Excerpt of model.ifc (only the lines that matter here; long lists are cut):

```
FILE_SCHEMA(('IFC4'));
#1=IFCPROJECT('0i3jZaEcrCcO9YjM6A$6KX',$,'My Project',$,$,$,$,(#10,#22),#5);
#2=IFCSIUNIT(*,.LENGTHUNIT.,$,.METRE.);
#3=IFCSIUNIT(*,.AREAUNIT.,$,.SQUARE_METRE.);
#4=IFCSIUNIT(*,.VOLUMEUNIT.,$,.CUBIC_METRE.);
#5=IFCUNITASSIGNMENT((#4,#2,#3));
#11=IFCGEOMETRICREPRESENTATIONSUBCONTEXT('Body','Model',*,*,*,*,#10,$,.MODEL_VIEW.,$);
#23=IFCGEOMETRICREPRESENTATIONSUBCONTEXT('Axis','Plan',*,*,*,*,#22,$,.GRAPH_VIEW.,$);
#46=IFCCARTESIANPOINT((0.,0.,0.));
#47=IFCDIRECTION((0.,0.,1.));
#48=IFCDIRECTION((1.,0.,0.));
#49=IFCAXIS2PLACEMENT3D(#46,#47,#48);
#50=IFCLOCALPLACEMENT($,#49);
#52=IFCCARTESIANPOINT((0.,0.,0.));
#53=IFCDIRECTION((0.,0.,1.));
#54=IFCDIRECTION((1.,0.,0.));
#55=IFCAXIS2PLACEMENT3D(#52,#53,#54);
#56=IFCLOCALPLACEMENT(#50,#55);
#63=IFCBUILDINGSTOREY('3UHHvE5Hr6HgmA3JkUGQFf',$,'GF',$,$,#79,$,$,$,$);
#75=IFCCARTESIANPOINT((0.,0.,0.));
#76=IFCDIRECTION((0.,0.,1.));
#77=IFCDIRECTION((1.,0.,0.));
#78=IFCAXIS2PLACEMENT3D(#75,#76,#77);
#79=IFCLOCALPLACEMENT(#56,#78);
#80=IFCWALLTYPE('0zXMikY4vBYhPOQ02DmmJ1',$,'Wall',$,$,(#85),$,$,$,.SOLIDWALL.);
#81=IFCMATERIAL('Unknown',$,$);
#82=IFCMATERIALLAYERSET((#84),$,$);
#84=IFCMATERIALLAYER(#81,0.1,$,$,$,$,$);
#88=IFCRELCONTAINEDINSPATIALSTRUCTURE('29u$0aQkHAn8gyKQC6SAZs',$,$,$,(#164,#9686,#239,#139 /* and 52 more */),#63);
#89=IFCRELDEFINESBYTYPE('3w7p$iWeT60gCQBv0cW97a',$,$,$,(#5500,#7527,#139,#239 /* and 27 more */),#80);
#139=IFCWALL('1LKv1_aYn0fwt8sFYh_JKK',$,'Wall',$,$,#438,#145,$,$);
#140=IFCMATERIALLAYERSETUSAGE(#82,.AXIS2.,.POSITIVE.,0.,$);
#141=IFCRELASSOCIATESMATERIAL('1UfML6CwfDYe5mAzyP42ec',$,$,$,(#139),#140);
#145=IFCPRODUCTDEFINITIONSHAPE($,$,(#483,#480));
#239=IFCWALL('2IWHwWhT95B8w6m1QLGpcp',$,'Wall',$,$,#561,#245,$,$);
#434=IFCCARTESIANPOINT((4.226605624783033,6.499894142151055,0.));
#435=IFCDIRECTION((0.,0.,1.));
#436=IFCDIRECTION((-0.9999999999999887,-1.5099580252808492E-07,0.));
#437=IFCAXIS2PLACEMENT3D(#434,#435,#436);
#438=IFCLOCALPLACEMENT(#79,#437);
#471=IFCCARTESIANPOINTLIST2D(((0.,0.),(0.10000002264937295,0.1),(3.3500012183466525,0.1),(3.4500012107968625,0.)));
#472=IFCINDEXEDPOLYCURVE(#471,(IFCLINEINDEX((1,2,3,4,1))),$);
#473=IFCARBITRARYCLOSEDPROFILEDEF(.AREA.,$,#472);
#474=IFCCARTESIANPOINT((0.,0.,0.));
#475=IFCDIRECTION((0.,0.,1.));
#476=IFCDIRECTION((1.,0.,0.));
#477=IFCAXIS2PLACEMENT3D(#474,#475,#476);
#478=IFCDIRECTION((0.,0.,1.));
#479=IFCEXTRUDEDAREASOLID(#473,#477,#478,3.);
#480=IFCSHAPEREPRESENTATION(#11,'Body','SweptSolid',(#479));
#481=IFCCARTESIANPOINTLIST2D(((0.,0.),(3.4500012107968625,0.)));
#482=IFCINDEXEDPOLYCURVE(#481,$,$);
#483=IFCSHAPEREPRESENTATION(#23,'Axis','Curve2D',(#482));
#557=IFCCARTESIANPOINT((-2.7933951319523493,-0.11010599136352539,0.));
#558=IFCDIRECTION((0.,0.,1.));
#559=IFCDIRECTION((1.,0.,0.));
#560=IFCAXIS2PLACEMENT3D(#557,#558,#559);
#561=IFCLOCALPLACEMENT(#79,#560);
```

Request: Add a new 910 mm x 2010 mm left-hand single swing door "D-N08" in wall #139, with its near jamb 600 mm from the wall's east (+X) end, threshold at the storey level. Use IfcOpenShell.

```python
import numpy as np
import ifcopenshell
import ifcopenshell.api.feature
import ifcopenshell.api.geometry
import ifcopenshell.api.root
import ifcopenshell.api.spatial
import ifcopenshell.geom
import ifcopenshell.util.element
import ifcopenshell.util.placement
import ifcopenshell.util.representation
import ifcopenshell.util.shape
import ifcopenshell.util.unit

model = ifcopenshell.open("model.ifc")
unit_scale = ifcopenshell.util.unit.calculate_unit_scale(model)
settings = ifcopenshell.geom.settings()


def volume(element):
    """Net volume in cubic metres, openings subtracted."""
    shape = ifcopenshell.geom.create_shape(settings, element)
    return ifcopenshell.util.shape.get_volume(shape.geometry)


wall = model.by_id(139)
storey = ifcopenshell.util.element.get_container(wall, ifc_class="IfcBuildingStorey")
context = ifcopenshell.util.representation.get_context(model, "Model", "Body", "MODEL_VIEW")
before = volume(wall)

width, height, from_end, sill = 0.91, 2.01, 0.6, 0.0  # metres

# The wall runs along its own X axis, and the end named is its -X end.
wall_shape = ifcopenshell.geom.create_shape(settings, wall)
x, y, z = ifcopenshell.util.shape.get_vertices(wall_shape.geometry).T
start = x.min() + from_end
face, thickness = float(y.min()), float(y.max() - y.min())
wall_matrix = ifcopenshell.util.placement.get_local_placement(wall.ObjectPlacement)
level = ifcopenshell.util.placement.get_local_placement(storey.ObjectPlacement)[2, 3]


def in_wall(x, y):
    """Placement at x, y metres in the wall's axes, at sill height."""
    matrix = wall_matrix.copy()
    matrix[:, 3] = wall_matrix @ np.array([x / unit_scale, y / unit_scale, 0.0, 1.0])
    matrix[2, 3] = level + sill / unit_scale
    return matrix


# Opening: a box that overshoots both wall faces by 50 mm.
opening = ifcopenshell.api.root.create_entity(model, ifc_class="IfcOpeningElement", predefined_type="OPENING")
box = ifcopenshell.api.geometry.add_wall_representation(
    model, context=context, length=width, height=height, thickness=thickness + 0.1
)
ifcopenshell.api.geometry.assign_representation(model, product=opening, representation=box)
ifcopenshell.api.geometry.edit_object_placement(model, product=opening, matrix=in_wall(start, face - 0.05), is_si=False)
ifcopenshell.api.feature.add_feature(model, feature=opening, element=wall)

door = ifcopenshell.api.root.create_entity(model, ifc_class="IfcDoor", name="D-N08", predefined_type="DOOR")
door.OverallWidth, door.OverallHeight = width / unit_scale, height / unit_scale
door.OperationType = "SINGLE_SWING_LEFT"
body = ifcopenshell.api.geometry.add_door_representation(
    model,
    context=context,
    overall_width=door.OverallWidth,
    overall_height=door.OverallHeight,
    operation_type="SINGLE_SWING_LEFT",
    lining_properties={"LiningDepth": thickness / unit_scale, "ThresholdDepth": thickness / unit_scale},
)
ifcopenshell.api.geometry.assign_representation(model, product=door, representation=body)
ifcopenshell.api.spatial.assign_container(model, products=[door], relating_structure=storey)
ifcopenshell.api.feature.add_filling(model, opening=opening, element=door)

# The lining spans the wall, so the door starts at the wall face.
ifcopenshell.api.geometry.edit_object_placement(model, product=door, matrix=in_wall(start, face), is_si=False)

after = volume(wall)

print(f"wall volume {before:.3f} -> {after:.3f} m3")

model.write("model_edited.ifc")
```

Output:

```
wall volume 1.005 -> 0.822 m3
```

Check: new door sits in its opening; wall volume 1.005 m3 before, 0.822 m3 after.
